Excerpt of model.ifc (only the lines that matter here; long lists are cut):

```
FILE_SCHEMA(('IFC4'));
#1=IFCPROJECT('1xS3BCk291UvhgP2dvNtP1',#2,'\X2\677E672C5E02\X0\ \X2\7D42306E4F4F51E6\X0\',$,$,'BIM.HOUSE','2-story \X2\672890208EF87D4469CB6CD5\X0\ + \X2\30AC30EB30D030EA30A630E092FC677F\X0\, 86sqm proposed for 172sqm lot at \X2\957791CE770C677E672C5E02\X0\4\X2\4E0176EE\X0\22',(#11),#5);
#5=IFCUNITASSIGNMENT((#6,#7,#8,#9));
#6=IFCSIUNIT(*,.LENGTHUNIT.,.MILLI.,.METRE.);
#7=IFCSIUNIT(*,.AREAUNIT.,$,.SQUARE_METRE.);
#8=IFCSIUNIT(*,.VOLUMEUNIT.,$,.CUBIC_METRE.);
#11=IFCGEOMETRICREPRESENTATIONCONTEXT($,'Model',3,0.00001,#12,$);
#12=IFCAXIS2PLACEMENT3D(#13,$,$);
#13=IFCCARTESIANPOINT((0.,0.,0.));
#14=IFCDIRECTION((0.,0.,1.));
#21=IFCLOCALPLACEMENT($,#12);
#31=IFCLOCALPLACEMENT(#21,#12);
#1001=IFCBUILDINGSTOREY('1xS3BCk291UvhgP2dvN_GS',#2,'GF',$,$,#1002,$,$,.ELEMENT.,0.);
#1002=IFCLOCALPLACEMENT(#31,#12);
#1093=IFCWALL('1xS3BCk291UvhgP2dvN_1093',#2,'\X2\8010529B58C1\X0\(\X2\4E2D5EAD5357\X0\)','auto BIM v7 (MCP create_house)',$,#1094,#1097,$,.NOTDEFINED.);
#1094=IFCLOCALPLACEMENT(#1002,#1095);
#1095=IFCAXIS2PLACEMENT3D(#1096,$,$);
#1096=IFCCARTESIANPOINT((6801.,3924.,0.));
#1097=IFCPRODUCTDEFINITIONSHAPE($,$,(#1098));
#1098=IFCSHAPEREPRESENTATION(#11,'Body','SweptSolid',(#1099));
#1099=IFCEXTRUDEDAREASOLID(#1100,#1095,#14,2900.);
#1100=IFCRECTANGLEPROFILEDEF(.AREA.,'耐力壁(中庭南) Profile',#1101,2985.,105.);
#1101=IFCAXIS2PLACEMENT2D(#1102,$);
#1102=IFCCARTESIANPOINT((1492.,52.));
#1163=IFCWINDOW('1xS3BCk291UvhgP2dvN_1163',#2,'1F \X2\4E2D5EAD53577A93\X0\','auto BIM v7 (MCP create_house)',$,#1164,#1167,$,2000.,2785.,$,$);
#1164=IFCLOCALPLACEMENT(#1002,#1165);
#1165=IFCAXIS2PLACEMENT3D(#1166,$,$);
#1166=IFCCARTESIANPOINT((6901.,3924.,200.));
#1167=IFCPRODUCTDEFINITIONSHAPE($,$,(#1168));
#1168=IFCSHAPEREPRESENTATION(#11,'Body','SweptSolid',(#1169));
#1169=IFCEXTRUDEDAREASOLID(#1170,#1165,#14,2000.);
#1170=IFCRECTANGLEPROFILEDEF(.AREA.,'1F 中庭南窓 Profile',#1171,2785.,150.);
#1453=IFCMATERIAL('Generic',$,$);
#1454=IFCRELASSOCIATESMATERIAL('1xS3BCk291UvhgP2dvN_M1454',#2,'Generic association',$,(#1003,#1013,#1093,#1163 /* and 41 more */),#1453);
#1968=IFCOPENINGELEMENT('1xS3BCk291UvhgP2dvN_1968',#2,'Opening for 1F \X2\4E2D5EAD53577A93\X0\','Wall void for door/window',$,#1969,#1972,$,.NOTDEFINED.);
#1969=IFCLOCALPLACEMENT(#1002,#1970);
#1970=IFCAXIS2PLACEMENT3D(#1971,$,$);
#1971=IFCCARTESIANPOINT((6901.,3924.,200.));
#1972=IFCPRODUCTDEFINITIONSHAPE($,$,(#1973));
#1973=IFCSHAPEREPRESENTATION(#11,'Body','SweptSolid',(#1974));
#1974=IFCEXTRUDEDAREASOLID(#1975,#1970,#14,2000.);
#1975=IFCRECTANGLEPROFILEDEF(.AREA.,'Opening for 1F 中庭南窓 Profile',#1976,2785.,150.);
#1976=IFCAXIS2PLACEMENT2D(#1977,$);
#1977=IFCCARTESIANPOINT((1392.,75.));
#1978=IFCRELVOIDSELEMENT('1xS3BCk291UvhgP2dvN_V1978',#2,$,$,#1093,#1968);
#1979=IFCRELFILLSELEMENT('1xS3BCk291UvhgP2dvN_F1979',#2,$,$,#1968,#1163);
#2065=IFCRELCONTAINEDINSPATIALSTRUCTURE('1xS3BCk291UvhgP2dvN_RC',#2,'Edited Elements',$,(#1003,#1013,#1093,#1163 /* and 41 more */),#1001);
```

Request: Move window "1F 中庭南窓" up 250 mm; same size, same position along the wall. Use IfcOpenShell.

```python
import numpy as np
import ifcopenshell
import ifcopenshell.api.geometry
import ifcopenshell.util.placement
import ifcopenshell.util.unit

model = ifcopenshell.open("model.ifc")
unit_scale = ifcopenshell.util.unit.calculate_unit_scale(model)

window = model.by_guid("1xS3BCk291UvhgP2dvN_1163")
opening = window.FillsVoids[0].RelatingOpeningElement
dz = 250.0

shift = np.array([0.0, 0.0, dz])
# The window is not placed relative to its opening, so move both.
for product in (opening, window):
    matrix = ifcopenshell.util.placement.get_local_placement(product.ObjectPlacement)
    matrix[:3, 3] += shift
    ifcopenshell.api.geometry.edit_object_placement(model, product=product, matrix=matrix, is_si=False)

print(f"moved by {dz * unit_scale:+.3f} m")

model.write("model_v2.ifc")
```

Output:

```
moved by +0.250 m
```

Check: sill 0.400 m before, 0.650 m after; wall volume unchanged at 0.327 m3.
